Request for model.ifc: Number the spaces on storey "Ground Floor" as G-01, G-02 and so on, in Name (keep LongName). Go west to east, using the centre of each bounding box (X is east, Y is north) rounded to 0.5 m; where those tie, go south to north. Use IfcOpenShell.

First a look at what the model holds.

```python
import ifcopenshell
import ifcopenshell.util.element
import ifcopenshell.util.placement

model = ifcopenshell.open("model.ifc")
print(model.schema)
storey = next(s for s in model.by_type("IfcBuildingStorey") if s.Name == "Ground Floor")
spaces = [e for e in ifcopenshell.util.element.get_decomposition(storey) if e.is_a("IfcSpace")]
for e in sorted(spaces, key=lambda e: e.id()):
    origin = ifcopenshell.util.placement.get_local_placement(e.ObjectPlacement)[:3, 3]
    print(e.id(), e.Name, e.LongName, origin.round(2) + 0.0, sep=" | ")
```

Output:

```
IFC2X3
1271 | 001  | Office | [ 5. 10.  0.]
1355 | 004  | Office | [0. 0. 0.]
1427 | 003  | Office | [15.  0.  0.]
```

```python
import ifcopenshell
import ifcopenshell.geom
import ifcopenshell.util.element
import ifcopenshell.util.shape

model = ifcopenshell.open("model.ifc")
settings = ifcopenshell.geom.settings()
settings.set("use-world-coords", True)


def centre(element):
    shape = ifcopenshell.geom.create_shape(settings, element)
    return ifcopenshell.util.shape.get_bbox_centroid(shape.geometry)


storey = next(s for s in model.by_type("IfcBuildingStorey") if s.Name == "Ground Floor")
spaces = [e for e in ifcopenshell.util.element.get_decomposition(storey) if e.is_a("IfcSpace")]

# Insertion points can sit at a corner or the storey origin, so sort by the geometry (in metres).
centres = {e: centre(e) for e in spaces}
spaces.sort(key=lambda e: (round(centres[e][0] / 0.5), centres[e][1]))

for i, e in enumerate(spaces, start=1):
    number = f"G-{i:02d}"
    e.Name = number
    print(e.id(), number)

model.write("model_rev.ifc")
```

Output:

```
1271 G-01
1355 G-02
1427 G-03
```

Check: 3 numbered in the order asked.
